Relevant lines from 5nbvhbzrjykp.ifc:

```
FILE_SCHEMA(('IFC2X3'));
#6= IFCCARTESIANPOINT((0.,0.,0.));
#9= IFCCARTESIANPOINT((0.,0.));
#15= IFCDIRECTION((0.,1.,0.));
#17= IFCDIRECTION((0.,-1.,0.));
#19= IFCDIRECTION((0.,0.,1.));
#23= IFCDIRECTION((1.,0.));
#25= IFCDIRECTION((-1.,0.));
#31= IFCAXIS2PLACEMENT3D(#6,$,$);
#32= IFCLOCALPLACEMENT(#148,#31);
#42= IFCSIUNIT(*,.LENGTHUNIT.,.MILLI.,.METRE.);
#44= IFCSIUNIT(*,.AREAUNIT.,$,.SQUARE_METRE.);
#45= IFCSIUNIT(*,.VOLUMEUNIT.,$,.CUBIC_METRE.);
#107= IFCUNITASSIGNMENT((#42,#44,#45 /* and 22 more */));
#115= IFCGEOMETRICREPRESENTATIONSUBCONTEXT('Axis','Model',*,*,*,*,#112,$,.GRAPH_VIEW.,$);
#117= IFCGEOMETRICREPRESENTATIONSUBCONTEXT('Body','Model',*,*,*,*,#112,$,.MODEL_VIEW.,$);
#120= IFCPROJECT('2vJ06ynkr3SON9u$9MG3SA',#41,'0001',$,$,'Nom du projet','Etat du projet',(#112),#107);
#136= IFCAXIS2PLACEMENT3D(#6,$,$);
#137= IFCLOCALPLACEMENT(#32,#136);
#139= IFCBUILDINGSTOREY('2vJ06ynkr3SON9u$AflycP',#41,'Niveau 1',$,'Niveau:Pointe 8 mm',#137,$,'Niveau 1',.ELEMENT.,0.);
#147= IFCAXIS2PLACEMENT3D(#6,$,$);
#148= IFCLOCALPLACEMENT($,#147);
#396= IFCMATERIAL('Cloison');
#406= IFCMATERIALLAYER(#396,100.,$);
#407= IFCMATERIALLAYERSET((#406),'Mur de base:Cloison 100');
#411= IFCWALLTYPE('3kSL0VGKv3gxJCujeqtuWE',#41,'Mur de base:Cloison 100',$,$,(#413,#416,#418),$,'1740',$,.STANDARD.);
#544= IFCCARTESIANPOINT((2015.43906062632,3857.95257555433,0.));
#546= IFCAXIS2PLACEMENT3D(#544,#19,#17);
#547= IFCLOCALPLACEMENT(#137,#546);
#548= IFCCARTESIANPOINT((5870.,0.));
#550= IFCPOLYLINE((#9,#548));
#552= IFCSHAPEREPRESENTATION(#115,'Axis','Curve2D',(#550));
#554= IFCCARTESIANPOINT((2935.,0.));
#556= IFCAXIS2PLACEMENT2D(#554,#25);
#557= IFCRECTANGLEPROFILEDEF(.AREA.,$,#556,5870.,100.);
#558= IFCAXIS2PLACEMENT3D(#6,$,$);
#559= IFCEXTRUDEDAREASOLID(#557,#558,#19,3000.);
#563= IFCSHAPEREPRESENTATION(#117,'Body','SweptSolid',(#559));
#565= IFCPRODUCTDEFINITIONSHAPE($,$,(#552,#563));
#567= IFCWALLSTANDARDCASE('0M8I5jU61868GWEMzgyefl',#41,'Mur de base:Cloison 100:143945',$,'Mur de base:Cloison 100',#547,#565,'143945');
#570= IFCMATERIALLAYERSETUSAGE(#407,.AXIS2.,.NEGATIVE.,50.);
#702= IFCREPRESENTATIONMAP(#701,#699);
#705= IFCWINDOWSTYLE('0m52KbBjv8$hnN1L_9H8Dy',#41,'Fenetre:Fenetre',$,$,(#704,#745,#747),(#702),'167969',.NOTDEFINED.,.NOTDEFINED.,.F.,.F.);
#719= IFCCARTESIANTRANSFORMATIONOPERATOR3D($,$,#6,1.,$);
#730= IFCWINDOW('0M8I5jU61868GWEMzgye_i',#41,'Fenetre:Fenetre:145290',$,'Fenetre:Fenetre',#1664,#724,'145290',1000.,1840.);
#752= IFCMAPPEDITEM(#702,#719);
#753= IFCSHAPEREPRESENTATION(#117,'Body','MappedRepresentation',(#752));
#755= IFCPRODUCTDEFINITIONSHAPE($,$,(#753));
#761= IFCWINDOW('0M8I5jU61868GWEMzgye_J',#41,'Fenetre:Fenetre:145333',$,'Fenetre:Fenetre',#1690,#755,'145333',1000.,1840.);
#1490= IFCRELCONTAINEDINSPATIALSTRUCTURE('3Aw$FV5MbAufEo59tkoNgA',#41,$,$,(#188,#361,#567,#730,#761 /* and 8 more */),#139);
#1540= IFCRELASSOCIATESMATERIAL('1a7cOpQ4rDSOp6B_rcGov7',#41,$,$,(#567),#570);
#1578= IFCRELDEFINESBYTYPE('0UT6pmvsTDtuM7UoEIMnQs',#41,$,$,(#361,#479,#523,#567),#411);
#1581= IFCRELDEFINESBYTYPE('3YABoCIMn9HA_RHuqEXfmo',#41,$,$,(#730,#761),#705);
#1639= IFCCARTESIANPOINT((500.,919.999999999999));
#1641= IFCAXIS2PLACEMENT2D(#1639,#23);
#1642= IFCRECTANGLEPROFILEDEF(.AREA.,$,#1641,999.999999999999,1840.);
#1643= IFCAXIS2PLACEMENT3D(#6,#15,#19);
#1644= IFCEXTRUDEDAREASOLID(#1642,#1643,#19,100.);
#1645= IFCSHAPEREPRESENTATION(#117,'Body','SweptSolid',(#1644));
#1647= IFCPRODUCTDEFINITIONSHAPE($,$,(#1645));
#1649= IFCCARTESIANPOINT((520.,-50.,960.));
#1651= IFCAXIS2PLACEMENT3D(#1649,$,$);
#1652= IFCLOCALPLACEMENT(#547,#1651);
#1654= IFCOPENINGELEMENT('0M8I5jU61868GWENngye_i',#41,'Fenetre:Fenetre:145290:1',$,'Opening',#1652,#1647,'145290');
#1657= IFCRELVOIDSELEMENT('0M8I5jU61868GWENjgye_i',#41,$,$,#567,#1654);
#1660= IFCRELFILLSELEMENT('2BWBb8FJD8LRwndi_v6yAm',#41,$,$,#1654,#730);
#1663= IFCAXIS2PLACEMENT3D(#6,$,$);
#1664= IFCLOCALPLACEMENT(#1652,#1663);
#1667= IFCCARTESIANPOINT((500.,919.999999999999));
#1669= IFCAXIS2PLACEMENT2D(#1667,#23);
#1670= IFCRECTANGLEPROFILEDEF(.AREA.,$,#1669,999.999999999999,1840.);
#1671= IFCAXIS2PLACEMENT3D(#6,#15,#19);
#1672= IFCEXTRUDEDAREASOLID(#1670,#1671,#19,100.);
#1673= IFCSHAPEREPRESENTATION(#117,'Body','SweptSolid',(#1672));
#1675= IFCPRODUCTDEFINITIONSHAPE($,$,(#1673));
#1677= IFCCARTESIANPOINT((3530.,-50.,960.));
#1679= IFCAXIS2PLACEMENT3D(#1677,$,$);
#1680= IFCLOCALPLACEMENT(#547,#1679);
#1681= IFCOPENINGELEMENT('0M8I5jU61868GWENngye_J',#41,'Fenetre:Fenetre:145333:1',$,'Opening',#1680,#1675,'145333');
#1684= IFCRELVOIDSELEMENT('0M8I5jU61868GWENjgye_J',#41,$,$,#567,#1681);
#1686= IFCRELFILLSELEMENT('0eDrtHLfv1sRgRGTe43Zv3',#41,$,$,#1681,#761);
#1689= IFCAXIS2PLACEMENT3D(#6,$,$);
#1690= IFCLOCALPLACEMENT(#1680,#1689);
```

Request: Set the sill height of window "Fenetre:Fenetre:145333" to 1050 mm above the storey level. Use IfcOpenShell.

```python
import numpy as np
import ifcopenshell
import ifcopenshell.api.geometry
import ifcopenshell.geom
import ifcopenshell.util.element
import ifcopenshell.util.placement
import ifcopenshell.util.shape
import ifcopenshell.util.unit

model = ifcopenshell.open("5nbvhbzrjykp.ifc")
unit_scale = ifcopenshell.util.unit.calculate_unit_scale(model)

window = model.by_guid("0M8I5jU61868GWEMzgye_J")
opening = window.FillsVoids[0].RelatingOpeningElement
storey = ifcopenshell.util.element.get_container(window, ifc_class="IfcBuildingStorey")
level = ifcopenshell.util.placement.get_local_placement(storey.ObjectPlacement)[2, 3]

# The opening's origin need not be at the sill, so measure its lowest point.
shape = ifcopenshell.geom.create_shape(ifcopenshell.geom.settings(), opening)
bottom = ifcopenshell.util.shape.get_shape_bottom_elevation(shape, shape.geometry) / unit_scale
dz = level + 1050.0 - bottom

shift = np.array([0.0, 0.0, dz])
# The window is placed relative to its opening, so it follows when the opening moves.
matrix = ifcopenshell.util.placement.get_local_placement(opening.ObjectPlacement)
matrix[:3, 3] += shift
ifcopenshell.api.geometry.edit_object_placement(
    model, product=opening, matrix=matrix, is_si=False, should_transform_children=True
)

print(f"moved by {dz * unit_scale:+.3f} m")

model.write("5nbvhbzrjykp_rev.ifc")
```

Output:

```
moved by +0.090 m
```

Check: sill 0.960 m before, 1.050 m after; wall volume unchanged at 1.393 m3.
